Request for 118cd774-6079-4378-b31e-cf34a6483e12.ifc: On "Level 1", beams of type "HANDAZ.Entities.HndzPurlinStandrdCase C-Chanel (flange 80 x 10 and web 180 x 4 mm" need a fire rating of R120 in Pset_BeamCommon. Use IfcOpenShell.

First a look at what the model holds.

```python
import ifcopenshell
import ifcopenshell.util.element

model = ifcopenshell.open("118cd774-6079-4378-b31e-cf34a6483e12.ifc")
print(model.schema)
storey = next(s for s in model.by_type("IfcBuildingStorey") if s.Name == "Level 1")
beams = [e for e in ifcopenshell.util.element.get_decomposition(storey) if e.is_a("IfcBeam")]
seen = {}
for e in beams:
    element_type = ifcopenshell.util.element.get_type(e)
    key = (element_type.Name if element_type != e and element_type else None, ifcopenshell.util.element.get_pset(e, "Pset_BeamCommon", "FireRating"))
    seen[key] = seen.get(key, 0) + 1
for (name, value), count in sorted(seen.items(), key=str):
    print(count, "x", name, "|", value)
```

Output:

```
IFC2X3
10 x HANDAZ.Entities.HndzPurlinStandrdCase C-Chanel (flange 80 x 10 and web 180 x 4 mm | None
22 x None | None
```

```python
import ifcopenshell
import ifcopenshell.api.pset
import ifcopenshell.util.element

model = ifcopenshell.open("118cd774-6079-4378-b31e-cf34a6483e12.ifc")

storey = next(s for s in model.by_type("IfcBuildingStorey") if s.Name == "Level 1")
beams = [e for e in ifcopenshell.util.element.get_decomposition(storey) if e.is_a("IfcBeam")]

count = 0
for e in beams:
    element_type = ifcopenshell.util.element.get_type(e)
    if element_type in (None, e) or element_type.Name != "HANDAZ.Entities.HndzPurlinStandrdCase C-Chanel (flange 80 x 10 and web 180 x 4 mm":
        continue
    # add_pset returns the element's existing set when there is one.
    pset = ifcopenshell.api.pset.add_pset(model, product=e, name="Pset_BeamCommon")
    ifcopenshell.api.pset.edit_pset(model, pset=pset, properties={"FireRating": "R120"})
    count += 1

print(count, "beams updated")

model.write("118cd774-6079-4378-b31e-cf34a6483e12_updated.ifc")
```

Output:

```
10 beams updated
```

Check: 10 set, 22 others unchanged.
